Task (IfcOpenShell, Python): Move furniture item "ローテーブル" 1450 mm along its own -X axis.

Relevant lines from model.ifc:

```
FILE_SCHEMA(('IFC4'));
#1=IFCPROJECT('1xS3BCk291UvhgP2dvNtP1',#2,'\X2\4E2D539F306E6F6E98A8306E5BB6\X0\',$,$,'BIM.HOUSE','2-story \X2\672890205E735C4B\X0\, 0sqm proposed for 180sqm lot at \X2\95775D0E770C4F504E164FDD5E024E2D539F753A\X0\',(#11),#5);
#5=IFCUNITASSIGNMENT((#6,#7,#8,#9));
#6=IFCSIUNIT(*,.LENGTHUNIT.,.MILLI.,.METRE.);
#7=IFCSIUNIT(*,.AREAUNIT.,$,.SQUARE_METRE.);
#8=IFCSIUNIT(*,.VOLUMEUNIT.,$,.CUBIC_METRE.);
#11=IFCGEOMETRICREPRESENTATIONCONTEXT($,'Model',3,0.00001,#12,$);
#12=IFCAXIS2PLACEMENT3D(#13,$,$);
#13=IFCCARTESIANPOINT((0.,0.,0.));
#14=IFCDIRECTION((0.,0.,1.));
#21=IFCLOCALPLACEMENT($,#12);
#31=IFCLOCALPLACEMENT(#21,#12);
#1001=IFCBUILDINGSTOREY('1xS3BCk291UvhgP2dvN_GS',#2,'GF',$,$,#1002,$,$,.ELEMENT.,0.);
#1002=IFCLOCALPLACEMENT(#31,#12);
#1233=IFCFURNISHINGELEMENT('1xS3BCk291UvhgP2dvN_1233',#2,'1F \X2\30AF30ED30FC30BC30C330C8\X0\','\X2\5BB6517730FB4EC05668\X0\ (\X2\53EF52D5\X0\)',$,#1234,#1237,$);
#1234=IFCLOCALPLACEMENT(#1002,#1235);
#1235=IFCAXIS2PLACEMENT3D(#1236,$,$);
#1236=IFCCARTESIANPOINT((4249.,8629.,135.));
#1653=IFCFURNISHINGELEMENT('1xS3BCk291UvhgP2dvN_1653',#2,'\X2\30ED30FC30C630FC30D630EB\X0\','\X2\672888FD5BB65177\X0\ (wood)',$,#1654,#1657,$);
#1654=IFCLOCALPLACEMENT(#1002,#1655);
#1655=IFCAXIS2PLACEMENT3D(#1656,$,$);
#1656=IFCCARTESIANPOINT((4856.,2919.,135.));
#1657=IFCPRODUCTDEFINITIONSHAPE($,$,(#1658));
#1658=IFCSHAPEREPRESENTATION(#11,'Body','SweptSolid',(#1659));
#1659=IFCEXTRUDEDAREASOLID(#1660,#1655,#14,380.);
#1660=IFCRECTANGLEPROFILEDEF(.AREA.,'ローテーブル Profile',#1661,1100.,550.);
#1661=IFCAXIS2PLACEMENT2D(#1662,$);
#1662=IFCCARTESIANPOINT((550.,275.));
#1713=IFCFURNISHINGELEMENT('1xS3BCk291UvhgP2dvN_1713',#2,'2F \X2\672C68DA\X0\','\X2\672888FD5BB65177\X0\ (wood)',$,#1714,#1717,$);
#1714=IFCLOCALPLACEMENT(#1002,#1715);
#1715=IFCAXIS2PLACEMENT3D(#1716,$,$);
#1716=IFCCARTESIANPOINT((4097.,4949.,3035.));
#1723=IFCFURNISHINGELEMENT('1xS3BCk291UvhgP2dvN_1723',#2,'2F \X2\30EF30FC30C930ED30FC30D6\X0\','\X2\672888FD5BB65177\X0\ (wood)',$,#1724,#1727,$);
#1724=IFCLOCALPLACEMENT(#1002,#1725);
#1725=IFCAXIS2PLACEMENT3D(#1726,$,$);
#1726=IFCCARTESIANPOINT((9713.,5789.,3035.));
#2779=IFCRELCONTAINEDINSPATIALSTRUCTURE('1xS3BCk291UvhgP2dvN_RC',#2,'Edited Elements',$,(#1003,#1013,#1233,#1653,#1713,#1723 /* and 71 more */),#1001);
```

```python
import ifcopenshell
import ifcopenshell.api.geometry
import ifcopenshell.util.placement

model = ifcopenshell.open("model.ifc")

item = model.by_id(1653)
matrix = ifcopenshell.util.placement.get_local_placement(item.ObjectPlacement)
matrix[:3, 3] -= matrix[:3, 0] * 1450.0
ifcopenshell.api.geometry.edit_object_placement(model, product=item, matrix=matrix, is_si=False)

print(ifcopenshell.util.placement.get_local_placement(item.ObjectPlacement).round(3) + 0.0)

model.write("model_updated.ifc")
```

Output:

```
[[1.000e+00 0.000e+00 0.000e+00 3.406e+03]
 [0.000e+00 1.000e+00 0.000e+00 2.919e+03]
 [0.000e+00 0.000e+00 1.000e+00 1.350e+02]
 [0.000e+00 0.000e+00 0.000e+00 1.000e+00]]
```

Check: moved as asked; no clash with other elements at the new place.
